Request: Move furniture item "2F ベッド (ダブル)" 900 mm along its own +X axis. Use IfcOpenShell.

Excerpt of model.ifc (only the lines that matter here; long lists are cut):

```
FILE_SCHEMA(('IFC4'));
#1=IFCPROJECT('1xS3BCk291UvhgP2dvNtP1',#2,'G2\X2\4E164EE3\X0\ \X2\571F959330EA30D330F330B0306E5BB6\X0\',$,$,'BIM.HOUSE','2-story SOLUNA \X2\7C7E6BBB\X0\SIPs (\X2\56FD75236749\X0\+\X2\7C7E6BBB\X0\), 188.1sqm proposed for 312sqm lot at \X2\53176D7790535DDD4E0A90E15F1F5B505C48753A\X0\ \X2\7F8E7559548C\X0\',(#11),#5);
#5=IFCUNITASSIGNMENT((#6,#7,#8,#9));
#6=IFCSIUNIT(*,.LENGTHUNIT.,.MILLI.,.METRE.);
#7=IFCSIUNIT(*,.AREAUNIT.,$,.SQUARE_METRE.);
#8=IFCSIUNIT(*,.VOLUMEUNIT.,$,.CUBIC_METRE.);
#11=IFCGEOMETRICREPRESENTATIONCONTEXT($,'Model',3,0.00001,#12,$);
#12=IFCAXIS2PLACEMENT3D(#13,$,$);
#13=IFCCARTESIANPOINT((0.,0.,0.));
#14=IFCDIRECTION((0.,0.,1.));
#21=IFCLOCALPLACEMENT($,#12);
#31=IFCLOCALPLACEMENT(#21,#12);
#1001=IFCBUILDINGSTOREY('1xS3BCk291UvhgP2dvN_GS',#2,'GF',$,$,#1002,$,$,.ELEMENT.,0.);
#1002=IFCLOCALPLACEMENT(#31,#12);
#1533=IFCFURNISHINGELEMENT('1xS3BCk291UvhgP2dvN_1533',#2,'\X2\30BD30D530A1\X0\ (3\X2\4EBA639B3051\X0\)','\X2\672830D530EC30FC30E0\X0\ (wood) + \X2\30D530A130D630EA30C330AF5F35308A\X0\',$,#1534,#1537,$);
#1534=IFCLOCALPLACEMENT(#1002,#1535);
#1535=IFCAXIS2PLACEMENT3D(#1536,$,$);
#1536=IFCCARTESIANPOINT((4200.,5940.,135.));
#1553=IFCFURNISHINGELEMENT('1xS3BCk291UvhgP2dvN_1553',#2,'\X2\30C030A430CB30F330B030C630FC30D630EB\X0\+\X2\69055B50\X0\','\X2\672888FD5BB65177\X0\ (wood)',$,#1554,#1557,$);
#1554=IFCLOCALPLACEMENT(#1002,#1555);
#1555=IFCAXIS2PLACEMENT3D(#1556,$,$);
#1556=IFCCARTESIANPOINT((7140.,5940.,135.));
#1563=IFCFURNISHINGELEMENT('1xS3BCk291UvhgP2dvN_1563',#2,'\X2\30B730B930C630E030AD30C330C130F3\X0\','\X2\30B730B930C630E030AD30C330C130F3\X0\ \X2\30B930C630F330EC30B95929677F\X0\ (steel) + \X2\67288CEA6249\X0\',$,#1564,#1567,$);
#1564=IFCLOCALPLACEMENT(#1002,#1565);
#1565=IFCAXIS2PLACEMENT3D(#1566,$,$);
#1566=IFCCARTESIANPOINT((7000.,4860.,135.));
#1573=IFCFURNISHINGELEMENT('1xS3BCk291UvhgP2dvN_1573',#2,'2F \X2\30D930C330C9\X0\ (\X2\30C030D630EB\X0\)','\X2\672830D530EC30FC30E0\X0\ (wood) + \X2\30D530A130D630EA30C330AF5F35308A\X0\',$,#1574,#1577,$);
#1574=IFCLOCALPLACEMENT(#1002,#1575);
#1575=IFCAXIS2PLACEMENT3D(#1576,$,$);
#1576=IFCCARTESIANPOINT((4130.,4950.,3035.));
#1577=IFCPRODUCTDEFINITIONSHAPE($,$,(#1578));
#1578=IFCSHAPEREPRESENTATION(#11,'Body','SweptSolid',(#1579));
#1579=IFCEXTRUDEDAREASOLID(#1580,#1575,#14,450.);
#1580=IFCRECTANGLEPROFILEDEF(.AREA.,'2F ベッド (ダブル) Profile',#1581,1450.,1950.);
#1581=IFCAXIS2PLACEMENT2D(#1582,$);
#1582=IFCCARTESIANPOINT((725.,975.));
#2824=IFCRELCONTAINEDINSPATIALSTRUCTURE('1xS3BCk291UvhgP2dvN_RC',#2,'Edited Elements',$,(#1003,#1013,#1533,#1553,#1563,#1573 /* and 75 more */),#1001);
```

```python
import ifcopenshell
import ifcopenshell.api.geometry
import ifcopenshell.util.placement

model = ifcopenshell.open("model.ifc")

item = model.by_guid("1xS3BCk291UvhgP2dvN_1573")
matrix = ifcopenshell.util.placement.get_local_placement(item.ObjectPlacement)
matrix[:3, 3] += matrix[:3, 0] * 900.0
ifcopenshell.api.geometry.edit_object_placement(model, product=item, matrix=matrix, is_si=False)

print(ifcopenshell.util.placement.get_local_placement(item.ObjectPlacement).round(3) + 0.0)

model.write("model-out.ifc")
```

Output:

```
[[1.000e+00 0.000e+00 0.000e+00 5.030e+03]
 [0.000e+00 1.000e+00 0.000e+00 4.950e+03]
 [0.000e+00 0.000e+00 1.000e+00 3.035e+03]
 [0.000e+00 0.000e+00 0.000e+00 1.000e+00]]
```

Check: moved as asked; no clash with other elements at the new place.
